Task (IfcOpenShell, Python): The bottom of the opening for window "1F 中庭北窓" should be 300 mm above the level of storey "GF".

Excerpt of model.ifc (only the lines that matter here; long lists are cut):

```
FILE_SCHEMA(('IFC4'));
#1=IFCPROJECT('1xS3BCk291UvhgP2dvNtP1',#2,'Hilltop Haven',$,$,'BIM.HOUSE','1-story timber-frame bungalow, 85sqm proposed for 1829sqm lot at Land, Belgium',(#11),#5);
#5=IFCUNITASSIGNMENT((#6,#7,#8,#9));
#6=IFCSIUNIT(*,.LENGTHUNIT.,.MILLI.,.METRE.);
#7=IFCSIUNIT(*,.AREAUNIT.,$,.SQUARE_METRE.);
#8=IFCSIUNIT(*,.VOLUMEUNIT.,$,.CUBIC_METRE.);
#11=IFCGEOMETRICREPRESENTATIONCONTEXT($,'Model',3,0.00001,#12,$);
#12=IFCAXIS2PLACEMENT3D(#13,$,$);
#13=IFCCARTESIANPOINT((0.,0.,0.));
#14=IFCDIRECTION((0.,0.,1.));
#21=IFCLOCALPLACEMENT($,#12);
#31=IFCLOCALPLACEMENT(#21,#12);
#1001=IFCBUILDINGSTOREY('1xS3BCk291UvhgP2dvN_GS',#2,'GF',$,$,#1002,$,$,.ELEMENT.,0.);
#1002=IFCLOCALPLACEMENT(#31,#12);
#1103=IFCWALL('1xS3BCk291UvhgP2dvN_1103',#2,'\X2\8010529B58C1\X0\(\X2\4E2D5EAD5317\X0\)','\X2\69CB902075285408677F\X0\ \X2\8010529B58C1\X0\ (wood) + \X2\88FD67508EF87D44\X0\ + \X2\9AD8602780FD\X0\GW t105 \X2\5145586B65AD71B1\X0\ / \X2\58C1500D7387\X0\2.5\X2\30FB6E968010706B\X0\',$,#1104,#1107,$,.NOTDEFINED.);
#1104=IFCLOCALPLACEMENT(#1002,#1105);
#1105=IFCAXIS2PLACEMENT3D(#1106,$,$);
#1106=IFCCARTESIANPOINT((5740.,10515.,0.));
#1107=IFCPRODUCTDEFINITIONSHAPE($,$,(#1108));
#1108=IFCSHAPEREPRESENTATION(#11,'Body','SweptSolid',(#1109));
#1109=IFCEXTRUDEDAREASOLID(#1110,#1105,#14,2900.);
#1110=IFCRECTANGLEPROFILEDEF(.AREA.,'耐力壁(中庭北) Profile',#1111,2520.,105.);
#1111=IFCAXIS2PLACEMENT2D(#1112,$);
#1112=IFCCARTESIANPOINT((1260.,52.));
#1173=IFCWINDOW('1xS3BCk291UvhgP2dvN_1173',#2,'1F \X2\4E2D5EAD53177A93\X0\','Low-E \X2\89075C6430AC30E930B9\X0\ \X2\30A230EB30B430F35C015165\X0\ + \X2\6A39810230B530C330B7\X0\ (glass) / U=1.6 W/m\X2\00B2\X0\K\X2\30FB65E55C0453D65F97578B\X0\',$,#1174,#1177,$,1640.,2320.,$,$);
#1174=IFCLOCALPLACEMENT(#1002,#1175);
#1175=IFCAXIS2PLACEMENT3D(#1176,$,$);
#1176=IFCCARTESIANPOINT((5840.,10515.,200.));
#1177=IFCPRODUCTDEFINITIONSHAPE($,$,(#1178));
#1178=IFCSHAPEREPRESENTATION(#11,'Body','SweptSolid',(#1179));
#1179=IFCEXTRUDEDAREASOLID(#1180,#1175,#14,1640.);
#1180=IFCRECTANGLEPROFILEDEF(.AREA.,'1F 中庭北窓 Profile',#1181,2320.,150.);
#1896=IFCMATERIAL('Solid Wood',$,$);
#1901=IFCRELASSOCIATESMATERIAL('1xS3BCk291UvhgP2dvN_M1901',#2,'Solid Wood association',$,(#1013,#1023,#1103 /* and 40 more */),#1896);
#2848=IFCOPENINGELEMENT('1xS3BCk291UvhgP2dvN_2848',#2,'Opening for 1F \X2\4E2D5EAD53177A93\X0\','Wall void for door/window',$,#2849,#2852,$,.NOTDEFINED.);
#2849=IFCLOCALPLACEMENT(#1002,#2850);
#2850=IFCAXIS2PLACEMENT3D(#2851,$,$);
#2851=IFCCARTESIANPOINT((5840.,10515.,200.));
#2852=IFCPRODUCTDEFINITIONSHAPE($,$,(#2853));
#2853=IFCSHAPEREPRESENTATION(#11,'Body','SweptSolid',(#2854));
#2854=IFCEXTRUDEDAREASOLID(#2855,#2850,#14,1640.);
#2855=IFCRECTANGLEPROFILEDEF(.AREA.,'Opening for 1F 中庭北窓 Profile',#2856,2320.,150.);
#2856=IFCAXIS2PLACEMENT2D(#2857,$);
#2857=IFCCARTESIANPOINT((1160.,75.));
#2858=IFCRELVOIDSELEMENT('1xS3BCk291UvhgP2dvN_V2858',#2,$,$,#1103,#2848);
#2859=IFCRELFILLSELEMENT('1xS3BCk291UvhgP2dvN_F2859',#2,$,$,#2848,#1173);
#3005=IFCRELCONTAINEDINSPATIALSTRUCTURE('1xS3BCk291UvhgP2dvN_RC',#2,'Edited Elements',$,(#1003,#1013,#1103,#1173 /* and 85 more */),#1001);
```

```python
import numpy as np
import ifcopenshell
import ifcopenshell.api.geometry
import ifcopenshell.geom
import ifcopenshell.util.element
import ifcopenshell.util.placement
import ifcopenshell.util.shape
import ifcopenshell.util.unit

model = ifcopenshell.open("model.ifc")
unit_scale = ifcopenshell.util.unit.calculate_unit_scale(model)

window = model.by_guid("1xS3BCk291UvhgP2dvN_1173")
opening = window.FillsVoids[0].RelatingOpeningElement
storey = ifcopenshell.util.element.get_container(window, ifc_class="IfcBuildingStorey")
level = ifcopenshell.util.placement.get_local_placement(storey.ObjectPlacement)[2, 3]

# The opening's origin need not be at the sill, so measure its lowest point.
shape = ifcopenshell.geom.create_shape(ifcopenshell.geom.settings(), opening)
bottom = ifcopenshell.util.shape.get_shape_bottom_elevation(shape, shape.geometry) / unit_scale
dz = level + 300.0 - bottom

shift = np.array([0.0, 0.0, dz])
# The window is not placed relative to its opening, so move both.
for product in (opening, window):
    matrix = ifcopenshell.util.placement.get_local_placement(product.ObjectPlacement)
    matrix[:3, 3] += shift
    ifcopenshell.api.geometry.edit_object_placement(model, product=product, matrix=matrix, is_si=False)

print(f"moved by {dz * unit_scale:+.3f} m")

model.write("model_rev.ifc")
```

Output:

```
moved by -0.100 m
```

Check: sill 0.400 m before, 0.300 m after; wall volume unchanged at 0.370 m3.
